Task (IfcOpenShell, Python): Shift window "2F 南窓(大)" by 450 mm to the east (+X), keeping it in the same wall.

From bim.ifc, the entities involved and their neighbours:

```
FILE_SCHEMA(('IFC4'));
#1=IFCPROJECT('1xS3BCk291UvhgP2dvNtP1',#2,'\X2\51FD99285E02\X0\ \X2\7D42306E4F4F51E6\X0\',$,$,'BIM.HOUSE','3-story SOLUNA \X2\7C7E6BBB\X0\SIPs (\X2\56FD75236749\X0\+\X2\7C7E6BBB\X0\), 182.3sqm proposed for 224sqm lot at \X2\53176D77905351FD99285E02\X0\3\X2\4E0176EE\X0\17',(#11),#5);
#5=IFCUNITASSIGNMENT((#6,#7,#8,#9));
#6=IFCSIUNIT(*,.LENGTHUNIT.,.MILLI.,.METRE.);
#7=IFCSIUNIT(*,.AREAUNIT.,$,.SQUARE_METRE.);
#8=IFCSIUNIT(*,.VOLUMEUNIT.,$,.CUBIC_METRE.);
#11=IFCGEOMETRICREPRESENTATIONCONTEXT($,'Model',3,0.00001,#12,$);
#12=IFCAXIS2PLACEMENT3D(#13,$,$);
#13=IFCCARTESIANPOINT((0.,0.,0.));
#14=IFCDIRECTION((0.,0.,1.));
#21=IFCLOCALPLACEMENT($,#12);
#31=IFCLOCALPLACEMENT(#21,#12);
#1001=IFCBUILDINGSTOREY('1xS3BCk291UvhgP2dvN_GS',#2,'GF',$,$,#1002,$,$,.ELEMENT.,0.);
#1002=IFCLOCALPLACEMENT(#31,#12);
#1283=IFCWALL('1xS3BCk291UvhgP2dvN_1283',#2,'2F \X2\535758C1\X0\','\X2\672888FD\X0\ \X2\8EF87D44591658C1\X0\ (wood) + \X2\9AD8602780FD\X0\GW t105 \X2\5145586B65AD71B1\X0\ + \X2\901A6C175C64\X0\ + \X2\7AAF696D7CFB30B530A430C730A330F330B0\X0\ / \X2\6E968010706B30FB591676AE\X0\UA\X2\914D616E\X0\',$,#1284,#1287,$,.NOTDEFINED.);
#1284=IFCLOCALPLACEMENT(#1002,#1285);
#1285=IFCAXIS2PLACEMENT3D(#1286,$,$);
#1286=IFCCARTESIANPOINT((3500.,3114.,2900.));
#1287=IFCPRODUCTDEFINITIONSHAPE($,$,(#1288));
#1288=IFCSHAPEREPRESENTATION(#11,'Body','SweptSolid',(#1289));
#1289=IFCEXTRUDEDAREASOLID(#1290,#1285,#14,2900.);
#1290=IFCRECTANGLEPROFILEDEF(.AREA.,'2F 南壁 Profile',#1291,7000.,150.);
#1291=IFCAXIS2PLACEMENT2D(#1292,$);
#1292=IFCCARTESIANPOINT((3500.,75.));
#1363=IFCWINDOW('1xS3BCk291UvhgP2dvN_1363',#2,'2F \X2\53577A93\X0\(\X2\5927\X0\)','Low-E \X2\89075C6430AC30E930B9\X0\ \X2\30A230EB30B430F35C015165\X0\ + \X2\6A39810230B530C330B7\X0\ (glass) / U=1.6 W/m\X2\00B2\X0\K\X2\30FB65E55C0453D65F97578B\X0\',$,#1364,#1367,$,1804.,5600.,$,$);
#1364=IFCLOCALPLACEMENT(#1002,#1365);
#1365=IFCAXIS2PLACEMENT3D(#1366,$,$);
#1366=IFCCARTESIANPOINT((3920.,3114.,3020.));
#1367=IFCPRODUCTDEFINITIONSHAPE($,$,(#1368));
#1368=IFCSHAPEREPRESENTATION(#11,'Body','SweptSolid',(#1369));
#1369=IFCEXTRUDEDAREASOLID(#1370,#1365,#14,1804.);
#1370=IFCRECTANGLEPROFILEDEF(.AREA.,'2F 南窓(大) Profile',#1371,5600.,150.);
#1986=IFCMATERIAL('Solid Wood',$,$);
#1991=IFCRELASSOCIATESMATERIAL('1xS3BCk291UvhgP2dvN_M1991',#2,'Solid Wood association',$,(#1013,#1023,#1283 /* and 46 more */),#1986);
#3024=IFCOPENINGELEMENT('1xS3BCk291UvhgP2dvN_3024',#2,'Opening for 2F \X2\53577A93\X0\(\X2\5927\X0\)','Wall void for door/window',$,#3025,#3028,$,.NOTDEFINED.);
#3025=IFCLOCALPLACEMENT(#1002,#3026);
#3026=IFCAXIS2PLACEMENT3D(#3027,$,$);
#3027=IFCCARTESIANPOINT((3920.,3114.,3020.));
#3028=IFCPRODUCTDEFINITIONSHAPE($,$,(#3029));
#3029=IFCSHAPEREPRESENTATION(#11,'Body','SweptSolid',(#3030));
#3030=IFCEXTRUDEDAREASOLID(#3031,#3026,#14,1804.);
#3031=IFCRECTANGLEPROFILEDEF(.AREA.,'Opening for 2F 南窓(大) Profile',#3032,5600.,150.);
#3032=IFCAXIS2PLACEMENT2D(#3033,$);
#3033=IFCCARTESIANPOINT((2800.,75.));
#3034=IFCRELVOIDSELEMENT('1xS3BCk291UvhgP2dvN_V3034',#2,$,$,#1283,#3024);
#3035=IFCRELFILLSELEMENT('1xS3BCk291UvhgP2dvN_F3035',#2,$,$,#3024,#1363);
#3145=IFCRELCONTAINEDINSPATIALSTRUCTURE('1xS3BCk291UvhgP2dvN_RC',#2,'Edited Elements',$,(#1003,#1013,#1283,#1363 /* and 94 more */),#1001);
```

```python
import ifcopenshell
import ifcopenshell.api.geometry
import ifcopenshell.util.placement
import ifcopenshell.util.unit

model = ifcopenshell.open("bim.ifc")
unit_scale = ifcopenshell.util.unit.calculate_unit_scale(model)

window = model.by_guid("1xS3BCk291UvhgP2dvN_1363")
opening = window.FillsVoids[0].RelatingOpeningElement
wall = opening.VoidsElements[0].RelatingBuildingElement

wall_matrix = ifcopenshell.util.placement.get_local_placement(wall.ObjectPlacement)
shift = wall_matrix[:3, 0] * 0.45 / unit_scale
before = ifcopenshell.util.placement.get_local_placement(window.ObjectPlacement)[:3, 3].copy()

# The window is not placed relative to its opening, so move both.
for product in (opening, window):
    matrix = ifcopenshell.util.placement.get_local_placement(product.ObjectPlacement)
    matrix[:3, 3] += shift
    ifcopenshell.api.geometry.edit_object_placement(model, product=product, matrix=matrix, is_si=False)

after = ifcopenshell.util.placement.get_local_placement(window.ObjectPlacement)[:3, 3]
print("window moved by", (after - before).round(3) + 0.0)

model.write("bim_rev.ifc")
```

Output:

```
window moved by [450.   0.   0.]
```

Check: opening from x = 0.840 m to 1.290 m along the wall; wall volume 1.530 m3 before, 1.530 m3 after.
